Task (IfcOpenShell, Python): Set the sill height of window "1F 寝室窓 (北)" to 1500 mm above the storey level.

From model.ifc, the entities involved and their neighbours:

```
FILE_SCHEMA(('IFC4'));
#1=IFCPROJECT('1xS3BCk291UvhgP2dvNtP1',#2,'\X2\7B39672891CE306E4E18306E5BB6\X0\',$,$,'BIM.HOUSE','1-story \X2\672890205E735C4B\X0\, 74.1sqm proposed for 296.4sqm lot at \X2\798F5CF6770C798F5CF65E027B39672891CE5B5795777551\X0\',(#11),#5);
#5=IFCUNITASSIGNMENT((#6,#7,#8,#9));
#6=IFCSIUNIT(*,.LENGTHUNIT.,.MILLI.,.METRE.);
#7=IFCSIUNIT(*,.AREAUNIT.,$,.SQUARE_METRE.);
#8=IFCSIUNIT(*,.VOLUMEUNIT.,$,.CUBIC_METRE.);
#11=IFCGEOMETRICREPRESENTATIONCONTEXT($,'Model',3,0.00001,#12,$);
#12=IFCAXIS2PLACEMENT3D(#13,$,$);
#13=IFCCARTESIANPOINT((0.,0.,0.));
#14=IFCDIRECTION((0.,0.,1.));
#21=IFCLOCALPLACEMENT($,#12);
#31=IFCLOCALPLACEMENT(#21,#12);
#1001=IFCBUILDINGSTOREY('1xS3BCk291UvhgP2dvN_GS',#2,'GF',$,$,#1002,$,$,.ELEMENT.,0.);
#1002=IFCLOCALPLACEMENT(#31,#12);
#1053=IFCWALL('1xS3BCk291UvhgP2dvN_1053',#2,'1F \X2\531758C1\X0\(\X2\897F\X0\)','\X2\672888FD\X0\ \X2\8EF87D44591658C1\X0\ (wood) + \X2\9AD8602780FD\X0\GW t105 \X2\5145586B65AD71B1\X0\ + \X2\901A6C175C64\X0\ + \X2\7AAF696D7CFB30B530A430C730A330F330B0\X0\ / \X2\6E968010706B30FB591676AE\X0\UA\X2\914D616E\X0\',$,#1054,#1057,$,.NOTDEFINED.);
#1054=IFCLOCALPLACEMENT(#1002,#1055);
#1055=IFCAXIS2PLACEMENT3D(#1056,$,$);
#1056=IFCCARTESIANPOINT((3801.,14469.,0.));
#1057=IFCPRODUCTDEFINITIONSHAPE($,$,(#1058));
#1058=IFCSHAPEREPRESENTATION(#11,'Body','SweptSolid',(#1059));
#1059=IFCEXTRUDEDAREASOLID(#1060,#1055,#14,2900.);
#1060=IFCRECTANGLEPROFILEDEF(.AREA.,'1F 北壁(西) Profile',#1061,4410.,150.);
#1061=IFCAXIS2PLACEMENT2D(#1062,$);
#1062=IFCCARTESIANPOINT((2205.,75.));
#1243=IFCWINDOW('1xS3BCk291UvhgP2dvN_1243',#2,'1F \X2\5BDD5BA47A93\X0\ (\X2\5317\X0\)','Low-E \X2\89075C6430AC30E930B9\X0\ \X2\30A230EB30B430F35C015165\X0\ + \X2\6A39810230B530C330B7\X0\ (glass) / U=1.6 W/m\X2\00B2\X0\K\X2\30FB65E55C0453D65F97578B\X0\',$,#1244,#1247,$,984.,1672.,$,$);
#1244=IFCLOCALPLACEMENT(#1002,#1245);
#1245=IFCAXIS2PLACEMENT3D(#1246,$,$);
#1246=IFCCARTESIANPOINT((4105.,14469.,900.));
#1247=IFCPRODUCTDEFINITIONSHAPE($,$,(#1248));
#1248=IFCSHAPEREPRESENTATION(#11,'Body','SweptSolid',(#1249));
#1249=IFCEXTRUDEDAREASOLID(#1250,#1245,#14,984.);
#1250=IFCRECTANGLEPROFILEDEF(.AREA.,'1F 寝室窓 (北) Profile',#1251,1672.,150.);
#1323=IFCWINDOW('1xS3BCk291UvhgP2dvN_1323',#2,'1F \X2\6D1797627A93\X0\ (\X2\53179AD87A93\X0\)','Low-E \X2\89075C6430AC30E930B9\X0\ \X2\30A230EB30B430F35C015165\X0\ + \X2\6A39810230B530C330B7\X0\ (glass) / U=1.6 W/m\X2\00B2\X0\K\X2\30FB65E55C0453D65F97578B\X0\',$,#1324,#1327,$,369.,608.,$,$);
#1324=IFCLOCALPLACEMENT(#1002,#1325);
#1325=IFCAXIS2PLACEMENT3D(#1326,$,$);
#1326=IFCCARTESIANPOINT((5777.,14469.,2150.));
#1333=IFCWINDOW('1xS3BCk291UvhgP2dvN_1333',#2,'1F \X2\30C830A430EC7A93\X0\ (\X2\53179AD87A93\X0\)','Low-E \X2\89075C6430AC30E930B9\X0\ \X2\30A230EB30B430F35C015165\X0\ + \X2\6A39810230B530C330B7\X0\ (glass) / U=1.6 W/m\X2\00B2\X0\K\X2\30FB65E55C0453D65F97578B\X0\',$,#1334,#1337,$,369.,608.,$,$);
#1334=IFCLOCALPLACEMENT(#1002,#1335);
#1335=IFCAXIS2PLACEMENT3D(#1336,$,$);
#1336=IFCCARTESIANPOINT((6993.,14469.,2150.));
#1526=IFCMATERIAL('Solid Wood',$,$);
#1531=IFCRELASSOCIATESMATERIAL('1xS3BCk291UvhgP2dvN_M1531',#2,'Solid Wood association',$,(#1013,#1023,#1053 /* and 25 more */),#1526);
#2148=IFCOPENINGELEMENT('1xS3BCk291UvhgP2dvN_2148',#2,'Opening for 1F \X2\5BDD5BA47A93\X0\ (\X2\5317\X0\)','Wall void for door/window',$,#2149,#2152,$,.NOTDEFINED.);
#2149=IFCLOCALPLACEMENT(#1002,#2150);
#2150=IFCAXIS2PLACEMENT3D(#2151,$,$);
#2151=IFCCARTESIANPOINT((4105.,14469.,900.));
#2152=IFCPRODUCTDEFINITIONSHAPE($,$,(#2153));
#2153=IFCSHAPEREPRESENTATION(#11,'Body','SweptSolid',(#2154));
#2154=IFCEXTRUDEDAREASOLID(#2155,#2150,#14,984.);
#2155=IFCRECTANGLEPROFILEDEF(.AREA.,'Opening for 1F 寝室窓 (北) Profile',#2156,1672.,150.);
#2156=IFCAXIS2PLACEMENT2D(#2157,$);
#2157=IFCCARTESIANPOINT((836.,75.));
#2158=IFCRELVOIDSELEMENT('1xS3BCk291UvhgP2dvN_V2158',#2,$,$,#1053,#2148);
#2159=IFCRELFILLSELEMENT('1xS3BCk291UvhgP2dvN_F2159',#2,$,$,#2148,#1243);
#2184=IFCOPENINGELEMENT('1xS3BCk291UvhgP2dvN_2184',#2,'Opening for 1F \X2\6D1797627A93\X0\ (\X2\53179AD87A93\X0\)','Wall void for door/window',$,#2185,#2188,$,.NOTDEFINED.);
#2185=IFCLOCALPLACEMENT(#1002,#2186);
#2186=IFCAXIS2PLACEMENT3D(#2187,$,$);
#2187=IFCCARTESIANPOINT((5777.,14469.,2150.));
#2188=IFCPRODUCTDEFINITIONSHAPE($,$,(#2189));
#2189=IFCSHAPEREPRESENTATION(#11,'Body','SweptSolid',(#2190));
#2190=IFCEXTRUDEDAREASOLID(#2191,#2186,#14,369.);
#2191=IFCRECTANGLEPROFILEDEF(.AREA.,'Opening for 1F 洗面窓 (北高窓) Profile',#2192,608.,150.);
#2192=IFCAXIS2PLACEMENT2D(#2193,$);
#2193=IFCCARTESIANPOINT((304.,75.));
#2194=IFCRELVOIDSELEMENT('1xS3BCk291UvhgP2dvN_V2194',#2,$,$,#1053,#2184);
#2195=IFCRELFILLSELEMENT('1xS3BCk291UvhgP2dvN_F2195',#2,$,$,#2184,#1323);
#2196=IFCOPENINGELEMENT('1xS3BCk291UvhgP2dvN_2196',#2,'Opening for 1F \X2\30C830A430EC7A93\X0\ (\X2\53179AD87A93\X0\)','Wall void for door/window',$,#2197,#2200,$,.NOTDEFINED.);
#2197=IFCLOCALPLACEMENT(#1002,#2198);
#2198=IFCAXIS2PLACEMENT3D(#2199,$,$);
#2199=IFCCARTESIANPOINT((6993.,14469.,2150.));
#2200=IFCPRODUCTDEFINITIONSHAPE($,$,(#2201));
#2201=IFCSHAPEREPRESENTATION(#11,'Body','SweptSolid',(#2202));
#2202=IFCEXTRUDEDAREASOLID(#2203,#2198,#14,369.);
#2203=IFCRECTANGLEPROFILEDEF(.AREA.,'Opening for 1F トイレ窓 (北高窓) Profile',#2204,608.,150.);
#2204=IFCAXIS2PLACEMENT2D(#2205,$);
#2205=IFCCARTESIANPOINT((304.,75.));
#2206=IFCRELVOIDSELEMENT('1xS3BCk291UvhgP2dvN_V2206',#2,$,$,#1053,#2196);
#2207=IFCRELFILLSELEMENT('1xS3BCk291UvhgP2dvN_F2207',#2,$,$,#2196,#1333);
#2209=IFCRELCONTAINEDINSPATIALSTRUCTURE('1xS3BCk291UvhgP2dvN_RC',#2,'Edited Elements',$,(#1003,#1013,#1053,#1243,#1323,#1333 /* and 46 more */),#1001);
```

```python
import numpy as np
import ifcopenshell
import ifcopenshell.api.geometry
import ifcopenshell.geom
import ifcopenshell.util.element
import ifcopenshell.util.placement
import ifcopenshell.util.shape
import ifcopenshell.util.unit

model = ifcopenshell.open("model.ifc")
unit_scale = ifcopenshell.util.unit.calculate_unit_scale(model)

window = model.by_guid("1xS3BCk291UvhgP2dvN_1243")
opening = window.FillsVoids[0].RelatingOpeningElement
storey = ifcopenshell.util.element.get_container(window, ifc_class="IfcBuildingStorey")
level = ifcopenshell.util.placement.get_local_placement(storey.ObjectPlacement)[2, 3]

# The opening's origin need not be at the sill, so measure its lowest point.
shape = ifcopenshell.geom.create_shape(ifcopenshell.geom.settings(), opening)
bottom = ifcopenshell.util.shape.get_shape_bottom_elevation(shape, shape.geometry) / unit_scale
dz = level + 1.5 / unit_scale - bottom

shift = np.array([0.0, 0.0, dz])
# The window is not placed relative to its opening, so move both.
for product in (opening, window):
    matrix = ifcopenshell.util.placement.get_local_placement(product.ObjectPlacement)
    matrix[:3, 3] += shift
    ifcopenshell.api.geometry.edit_object_placement(model, product=product, matrix=matrix, is_si=False)

print(f"moved by {dz * unit_scale:+.3f} m")

model.write("model_v2.ifc")
```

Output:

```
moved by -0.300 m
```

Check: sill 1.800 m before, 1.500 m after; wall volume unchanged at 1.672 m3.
